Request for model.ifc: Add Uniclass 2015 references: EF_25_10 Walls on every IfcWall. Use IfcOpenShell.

First a look at what the model holds.

```python
import ifcopenshell

model = ifcopenshell.open("model.ifc")
print(model.schema)
print("classifications:", [c.Name for c in model.by_type("IfcClassification")])
for ifc_class in ("IfcDoor", "IfcRoof", "IfcStair", "IfcWall", "IfcWindow"):
    print(ifc_class, len(model.by_type(ifc_class)))
```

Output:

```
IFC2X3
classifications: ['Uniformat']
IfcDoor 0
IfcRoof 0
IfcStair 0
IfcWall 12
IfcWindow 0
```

```python
import ifcopenshell
import ifcopenshell.api.classification

model = ifcopenshell.open("model.ifc")

# IFC2X3 requires Source and Edition and has no link from the project to the system.
system = model.create_entity("IfcClassification", Source="NBS", Edition="2015", Name="Uniclass 2015")

codes = {
    "IfcWall": ("EF_25_10", "Walls"),
}
for ifc_class, (code, name) in codes.items():
    products = model.by_type(ifc_class)
    ifcopenshell.api.classification.add_reference(
        model, products=products, classification=system, identification=code, name=name
    )
    print(code, len(products))

model.write("model_rev.ifc")
```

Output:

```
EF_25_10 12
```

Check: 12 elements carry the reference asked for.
